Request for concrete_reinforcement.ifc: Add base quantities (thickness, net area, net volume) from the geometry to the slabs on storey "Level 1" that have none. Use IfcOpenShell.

First a look at what the model holds.

```python
import ifcopenshell
import ifcopenshell.util.element
import ifcopenshell.util.unit

model = ifcopenshell.open("concrete_reinforcement.ifc")
print(model.schema)
for unit_type in ("LENGTHUNIT", "AREAUNIT", "VOLUMEUNIT"):
    print(unit_type, ifcopenshell.util.unit.calculate_unit_scale(model, unit_type))
storey = next(s for s in model.by_type("IfcBuildingStorey") if s.Name == "Level 1")
slabs = [e for e in ifcopenshell.util.element.get_decomposition(storey) if e.is_a("IfcSlab")]
for e in sorted(slabs, key=lambda e: e.id()):
    print(e.id(), e.is_a(), e.Name, list(ifcopenshell.util.element.get_psets(e, qtos_only=True)), sep=" | ")
```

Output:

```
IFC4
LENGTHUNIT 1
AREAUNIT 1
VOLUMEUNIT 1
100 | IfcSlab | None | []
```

```python
import ifcopenshell
import ifcopenshell.api.pset
import ifcopenshell.geom
import ifcopenshell.util.element
import ifcopenshell.util.shape
import ifcopenshell.util.unit

model = ifcopenshell.open("concrete_reinforcement.ifc")
unit_scale = ifcopenshell.util.unit.calculate_unit_scale(model)
area_scale = ifcopenshell.util.unit.calculate_unit_scale(model, "AREAUNIT")
volume_scale = ifcopenshell.util.unit.calculate_unit_scale(model, "VOLUMEUNIT")
settings = ifcopenshell.geom.settings()

storey = next(s for s in model.by_type("IfcBuildingStorey") if s.Name == "Level 1")
slabs = [e for e in ifcopenshell.util.element.get_decomposition(storey) if e.is_a("IfcSlab")]

for e in sorted(slabs, key=lambda e: e.id()):
    if ifcopenshell.util.element.get_psets(e, qtos_only=True, should_inherit=False):
        continue
    # Geometry comes back in metres, in the element's own axes.
    shape = ifcopenshell.geom.create_shape(settings, e)
    values = {
        "Width": ifcopenshell.util.shape.get_z(shape.geometry) / unit_scale,
        "NetArea": ifcopenshell.util.shape.get_footprint_area(shape.geometry) / area_scale,
        "NetVolume": ifcopenshell.util.shape.get_volume(shape.geometry) / volume_scale,
    }
    qto = ifcopenshell.api.pset.add_qto(model, product=e, name="Qto_SlabBaseQuantities")
    ifcopenshell.api.pset.edit_qto(model, qto=qto, properties=values)
    print(e.id(), {k: round(v, 3) for k, v in values.items()})

model.write("concrete_reinforcement-out.ifc")
```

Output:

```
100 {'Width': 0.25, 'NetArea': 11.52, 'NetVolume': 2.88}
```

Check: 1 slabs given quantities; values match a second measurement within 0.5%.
